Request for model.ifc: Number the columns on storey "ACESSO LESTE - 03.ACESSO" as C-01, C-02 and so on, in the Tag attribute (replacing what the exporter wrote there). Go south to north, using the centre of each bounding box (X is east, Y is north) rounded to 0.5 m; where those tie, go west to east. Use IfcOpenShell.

First a look at what the model holds.

```python
import ifcopenshell
import ifcopenshell.util.element
import ifcopenshell.util.placement

model = ifcopenshell.open("model.ifc")
print(model.schema)
storey = next(s for s in model.by_type("IfcBuildingStorey") if s.Name == "ACESSO LESTE - 03.ACESSO")
columns = [e for e in ifcopenshell.util.element.get_decomposition(storey) if e.is_a("IfcColumn")]
for e in sorted(columns, key=lambda e: e.id()):
    origin = ifcopenshell.util.placement.get_local_placement(e.ObjectPlacement)[:3, 3]
    print(e.id(), e.Tag, e.Name, origin.round(2) + 0.0, sep=" | ")
```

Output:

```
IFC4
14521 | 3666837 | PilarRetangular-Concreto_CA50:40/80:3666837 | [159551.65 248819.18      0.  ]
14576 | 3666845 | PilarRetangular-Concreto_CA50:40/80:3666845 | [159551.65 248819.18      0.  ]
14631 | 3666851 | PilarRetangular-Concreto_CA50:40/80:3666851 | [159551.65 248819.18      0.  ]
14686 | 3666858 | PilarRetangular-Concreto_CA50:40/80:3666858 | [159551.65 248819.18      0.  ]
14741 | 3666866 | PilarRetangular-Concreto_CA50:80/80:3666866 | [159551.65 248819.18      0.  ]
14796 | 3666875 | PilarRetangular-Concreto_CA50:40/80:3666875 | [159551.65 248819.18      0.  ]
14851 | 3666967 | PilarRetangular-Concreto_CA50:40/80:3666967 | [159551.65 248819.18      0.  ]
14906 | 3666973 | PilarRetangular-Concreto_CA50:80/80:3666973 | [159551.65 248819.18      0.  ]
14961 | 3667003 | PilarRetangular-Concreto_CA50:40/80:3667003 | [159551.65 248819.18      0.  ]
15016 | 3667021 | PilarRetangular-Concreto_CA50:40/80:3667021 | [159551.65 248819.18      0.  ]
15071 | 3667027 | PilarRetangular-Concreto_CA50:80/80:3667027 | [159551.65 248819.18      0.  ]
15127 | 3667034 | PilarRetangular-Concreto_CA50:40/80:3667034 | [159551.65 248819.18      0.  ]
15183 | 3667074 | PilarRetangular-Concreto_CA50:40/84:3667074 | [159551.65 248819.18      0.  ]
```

```python
import ifcopenshell
import ifcopenshell.geom
import ifcopenshell.util.element
import ifcopenshell.util.shape

model = ifcopenshell.open("model.ifc")
settings = ifcopenshell.geom.settings()
settings.set("use-world-coords", True)


def centre(element):
    shape = ifcopenshell.geom.create_shape(settings, element)
    return ifcopenshell.util.shape.get_bbox_centroid(shape.geometry)


storey = next(s for s in model.by_type("IfcBuildingStorey") if s.Name == "ACESSO LESTE - 03.ACESSO")
columns = [e for e in ifcopenshell.util.element.get_decomposition(storey) if e.is_a("IfcColumn")]

# Insertion points can sit at a corner or the storey origin, so sort by the geometry (in metres).
centres = {e: centre(e) for e in columns}
columns.sort(key=lambda e: (round(centres[e][1] / 0.5), centres[e][0]))

for i, e in enumerate(columns, start=1):
    number = f"C-{i:02d}"
    e.Tag = number
    print(e.id(), number)

model.write("model_updated.ifc")
```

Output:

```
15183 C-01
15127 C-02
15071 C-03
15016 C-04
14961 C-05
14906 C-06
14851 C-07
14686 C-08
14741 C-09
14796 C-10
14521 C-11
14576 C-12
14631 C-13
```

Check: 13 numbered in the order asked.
